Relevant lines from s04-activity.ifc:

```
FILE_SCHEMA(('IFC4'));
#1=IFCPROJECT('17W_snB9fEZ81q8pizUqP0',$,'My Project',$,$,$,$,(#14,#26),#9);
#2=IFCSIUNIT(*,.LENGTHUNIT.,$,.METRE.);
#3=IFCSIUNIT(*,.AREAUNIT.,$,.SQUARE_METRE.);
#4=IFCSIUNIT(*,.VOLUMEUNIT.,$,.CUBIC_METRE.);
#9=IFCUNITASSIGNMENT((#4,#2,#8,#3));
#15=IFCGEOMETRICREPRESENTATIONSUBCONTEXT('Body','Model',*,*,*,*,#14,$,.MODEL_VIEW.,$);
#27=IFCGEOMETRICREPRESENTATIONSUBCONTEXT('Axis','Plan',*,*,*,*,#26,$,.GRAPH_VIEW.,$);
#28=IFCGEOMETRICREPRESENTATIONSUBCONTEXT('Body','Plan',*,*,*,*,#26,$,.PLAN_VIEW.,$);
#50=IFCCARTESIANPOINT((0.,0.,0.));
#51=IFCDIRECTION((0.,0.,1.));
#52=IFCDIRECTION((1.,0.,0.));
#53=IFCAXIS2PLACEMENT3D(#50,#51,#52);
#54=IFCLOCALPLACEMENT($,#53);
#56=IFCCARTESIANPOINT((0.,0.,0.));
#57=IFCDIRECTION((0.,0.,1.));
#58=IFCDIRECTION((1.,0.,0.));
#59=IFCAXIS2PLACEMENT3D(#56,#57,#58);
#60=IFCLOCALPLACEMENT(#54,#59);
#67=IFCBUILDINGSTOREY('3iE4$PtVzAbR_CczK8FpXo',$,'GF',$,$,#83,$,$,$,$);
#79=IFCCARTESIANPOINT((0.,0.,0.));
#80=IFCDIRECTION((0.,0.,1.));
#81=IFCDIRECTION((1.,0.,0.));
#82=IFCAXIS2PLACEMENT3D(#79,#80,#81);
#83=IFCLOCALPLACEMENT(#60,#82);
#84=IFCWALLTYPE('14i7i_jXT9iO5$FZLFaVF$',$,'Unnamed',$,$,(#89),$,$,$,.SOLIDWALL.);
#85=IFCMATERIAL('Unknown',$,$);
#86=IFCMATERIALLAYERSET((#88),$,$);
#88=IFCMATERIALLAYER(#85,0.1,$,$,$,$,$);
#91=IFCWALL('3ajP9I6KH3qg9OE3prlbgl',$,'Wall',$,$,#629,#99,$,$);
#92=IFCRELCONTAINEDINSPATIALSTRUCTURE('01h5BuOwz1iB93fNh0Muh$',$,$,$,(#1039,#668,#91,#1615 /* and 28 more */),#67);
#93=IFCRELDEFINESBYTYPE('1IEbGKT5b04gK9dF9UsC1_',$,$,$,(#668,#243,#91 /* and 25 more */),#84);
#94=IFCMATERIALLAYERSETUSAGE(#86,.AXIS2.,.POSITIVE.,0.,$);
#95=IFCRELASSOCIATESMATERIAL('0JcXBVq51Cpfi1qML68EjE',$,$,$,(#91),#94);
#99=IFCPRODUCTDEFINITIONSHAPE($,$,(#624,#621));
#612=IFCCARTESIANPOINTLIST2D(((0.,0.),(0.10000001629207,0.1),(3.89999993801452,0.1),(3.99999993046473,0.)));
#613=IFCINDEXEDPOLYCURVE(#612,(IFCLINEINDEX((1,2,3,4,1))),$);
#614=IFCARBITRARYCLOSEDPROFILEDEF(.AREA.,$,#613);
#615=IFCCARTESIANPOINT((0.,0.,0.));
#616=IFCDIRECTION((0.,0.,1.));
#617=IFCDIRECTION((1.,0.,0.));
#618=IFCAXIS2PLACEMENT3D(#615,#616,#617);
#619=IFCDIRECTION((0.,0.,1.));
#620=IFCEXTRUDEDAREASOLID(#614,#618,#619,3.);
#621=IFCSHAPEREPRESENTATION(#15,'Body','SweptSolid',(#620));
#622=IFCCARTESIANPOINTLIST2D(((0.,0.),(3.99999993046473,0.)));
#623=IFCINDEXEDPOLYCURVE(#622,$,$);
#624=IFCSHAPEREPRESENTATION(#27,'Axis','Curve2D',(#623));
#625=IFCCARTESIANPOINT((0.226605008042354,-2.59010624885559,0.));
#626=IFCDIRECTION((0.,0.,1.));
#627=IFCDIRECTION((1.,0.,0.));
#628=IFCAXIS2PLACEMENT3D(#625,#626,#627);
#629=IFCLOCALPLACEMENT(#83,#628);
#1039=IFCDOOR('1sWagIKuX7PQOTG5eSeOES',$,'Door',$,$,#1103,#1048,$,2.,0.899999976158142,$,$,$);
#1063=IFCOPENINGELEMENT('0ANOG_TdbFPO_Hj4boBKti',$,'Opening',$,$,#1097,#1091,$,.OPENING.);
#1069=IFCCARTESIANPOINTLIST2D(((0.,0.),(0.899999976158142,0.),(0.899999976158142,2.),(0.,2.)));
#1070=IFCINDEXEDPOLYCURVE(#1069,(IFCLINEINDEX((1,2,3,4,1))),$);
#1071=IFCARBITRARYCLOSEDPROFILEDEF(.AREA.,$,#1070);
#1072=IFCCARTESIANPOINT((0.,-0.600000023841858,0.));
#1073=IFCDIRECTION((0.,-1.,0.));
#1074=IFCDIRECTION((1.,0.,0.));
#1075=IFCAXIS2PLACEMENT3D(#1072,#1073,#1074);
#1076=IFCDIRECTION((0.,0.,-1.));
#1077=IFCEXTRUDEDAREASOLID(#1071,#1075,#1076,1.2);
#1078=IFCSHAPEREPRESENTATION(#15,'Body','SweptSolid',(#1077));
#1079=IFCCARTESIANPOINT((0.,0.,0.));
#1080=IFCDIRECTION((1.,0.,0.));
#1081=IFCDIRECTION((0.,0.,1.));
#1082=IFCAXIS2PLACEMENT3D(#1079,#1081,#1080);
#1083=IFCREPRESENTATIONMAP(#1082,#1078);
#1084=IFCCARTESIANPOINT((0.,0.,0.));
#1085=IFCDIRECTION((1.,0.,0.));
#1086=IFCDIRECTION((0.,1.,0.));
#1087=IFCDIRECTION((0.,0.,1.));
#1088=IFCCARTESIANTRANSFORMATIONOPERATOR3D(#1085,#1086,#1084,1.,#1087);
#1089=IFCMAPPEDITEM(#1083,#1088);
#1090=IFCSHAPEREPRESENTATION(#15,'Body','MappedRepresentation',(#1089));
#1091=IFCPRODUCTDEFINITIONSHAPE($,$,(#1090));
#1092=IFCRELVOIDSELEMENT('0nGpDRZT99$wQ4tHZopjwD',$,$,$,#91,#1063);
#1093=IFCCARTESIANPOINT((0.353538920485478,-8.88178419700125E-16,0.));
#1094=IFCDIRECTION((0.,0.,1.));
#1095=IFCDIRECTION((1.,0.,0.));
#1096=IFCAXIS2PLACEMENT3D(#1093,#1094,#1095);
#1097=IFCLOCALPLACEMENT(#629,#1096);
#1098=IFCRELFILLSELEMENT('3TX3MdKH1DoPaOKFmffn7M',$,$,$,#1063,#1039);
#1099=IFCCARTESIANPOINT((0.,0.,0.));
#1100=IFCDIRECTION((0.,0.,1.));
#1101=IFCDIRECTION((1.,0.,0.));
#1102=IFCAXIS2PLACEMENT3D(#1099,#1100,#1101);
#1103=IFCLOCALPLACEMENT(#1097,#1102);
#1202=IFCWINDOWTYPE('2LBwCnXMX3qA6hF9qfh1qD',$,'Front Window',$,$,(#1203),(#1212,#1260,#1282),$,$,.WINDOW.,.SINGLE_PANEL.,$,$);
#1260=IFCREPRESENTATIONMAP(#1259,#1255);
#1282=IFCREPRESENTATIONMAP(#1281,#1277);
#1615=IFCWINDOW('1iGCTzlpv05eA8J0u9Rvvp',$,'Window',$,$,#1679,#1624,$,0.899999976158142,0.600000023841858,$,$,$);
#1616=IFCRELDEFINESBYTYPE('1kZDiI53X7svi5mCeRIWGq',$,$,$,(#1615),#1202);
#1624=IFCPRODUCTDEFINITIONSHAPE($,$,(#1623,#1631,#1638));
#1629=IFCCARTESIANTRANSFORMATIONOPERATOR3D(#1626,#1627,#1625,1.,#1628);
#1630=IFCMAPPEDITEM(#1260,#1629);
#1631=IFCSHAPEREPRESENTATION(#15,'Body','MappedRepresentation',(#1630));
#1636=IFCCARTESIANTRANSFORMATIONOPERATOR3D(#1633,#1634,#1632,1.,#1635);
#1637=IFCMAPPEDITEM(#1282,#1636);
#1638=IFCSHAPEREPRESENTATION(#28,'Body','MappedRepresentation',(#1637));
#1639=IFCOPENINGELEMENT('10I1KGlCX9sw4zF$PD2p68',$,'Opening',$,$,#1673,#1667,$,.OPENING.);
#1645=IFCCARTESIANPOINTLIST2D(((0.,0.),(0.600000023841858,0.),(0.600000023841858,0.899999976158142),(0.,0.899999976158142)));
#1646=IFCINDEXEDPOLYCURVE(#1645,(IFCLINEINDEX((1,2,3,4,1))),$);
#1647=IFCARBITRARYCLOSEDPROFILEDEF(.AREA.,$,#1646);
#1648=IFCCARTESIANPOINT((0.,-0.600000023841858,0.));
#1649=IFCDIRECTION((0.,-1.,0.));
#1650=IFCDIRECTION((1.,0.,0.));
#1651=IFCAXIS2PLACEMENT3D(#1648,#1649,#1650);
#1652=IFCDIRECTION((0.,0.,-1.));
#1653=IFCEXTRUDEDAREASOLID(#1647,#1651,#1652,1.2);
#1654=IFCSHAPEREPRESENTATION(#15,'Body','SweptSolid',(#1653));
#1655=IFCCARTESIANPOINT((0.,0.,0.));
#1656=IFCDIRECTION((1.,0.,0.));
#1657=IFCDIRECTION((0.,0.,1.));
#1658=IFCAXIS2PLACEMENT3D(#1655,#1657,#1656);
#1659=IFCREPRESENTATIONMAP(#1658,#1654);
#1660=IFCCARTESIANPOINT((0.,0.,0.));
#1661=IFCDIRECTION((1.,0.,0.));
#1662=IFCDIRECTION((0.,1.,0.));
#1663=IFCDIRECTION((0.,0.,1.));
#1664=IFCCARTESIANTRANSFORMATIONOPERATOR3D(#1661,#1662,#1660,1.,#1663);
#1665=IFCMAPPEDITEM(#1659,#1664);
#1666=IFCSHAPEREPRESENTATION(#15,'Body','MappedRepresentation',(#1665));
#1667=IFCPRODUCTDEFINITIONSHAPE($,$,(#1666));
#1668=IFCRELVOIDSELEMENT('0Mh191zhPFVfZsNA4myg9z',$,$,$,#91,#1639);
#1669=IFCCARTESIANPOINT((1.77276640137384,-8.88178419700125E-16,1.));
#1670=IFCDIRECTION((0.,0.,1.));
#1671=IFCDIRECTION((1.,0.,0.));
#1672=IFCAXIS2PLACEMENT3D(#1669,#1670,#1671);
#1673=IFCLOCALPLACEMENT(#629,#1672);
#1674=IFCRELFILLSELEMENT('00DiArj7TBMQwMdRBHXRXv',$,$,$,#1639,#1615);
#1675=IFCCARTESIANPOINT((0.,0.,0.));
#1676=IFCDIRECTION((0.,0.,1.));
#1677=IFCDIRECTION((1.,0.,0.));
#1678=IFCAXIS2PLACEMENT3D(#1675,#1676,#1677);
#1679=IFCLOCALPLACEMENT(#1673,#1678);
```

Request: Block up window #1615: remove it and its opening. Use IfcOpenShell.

```python
import ifcopenshell
import ifcopenshell.api.feature
import ifcopenshell.api.root
import ifcopenshell.geom
import ifcopenshell.util.shape

model = ifcopenshell.open("s04-activity.ifc")
settings = ifcopenshell.geom.settings()


def volume(element):
    """Net volume in cubic metres, openings subtracted."""
    shape = ifcopenshell.geom.create_shape(settings, element)
    return ifcopenshell.util.shape.get_volume(shape.geometry)


window = model.by_guid("1iGCTzlpv05eA8J0u9Rvvp")
opening = window.FillsVoids[0].RelatingOpeningElement
wall = opening.VoidsElements[0].RelatingBuildingElement
before = volume(wall)

ifcopenshell.api.root.remove_product(model, product=window)
ifcopenshell.api.feature.remove_feature(model, feature=opening)

after = volume(wall)

print(f"wall volume {before:.3f} -> {after:.3f} m3")

model.write("s04-activity_v2.ifc")
```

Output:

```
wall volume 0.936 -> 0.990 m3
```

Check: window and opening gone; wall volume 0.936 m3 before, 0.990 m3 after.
